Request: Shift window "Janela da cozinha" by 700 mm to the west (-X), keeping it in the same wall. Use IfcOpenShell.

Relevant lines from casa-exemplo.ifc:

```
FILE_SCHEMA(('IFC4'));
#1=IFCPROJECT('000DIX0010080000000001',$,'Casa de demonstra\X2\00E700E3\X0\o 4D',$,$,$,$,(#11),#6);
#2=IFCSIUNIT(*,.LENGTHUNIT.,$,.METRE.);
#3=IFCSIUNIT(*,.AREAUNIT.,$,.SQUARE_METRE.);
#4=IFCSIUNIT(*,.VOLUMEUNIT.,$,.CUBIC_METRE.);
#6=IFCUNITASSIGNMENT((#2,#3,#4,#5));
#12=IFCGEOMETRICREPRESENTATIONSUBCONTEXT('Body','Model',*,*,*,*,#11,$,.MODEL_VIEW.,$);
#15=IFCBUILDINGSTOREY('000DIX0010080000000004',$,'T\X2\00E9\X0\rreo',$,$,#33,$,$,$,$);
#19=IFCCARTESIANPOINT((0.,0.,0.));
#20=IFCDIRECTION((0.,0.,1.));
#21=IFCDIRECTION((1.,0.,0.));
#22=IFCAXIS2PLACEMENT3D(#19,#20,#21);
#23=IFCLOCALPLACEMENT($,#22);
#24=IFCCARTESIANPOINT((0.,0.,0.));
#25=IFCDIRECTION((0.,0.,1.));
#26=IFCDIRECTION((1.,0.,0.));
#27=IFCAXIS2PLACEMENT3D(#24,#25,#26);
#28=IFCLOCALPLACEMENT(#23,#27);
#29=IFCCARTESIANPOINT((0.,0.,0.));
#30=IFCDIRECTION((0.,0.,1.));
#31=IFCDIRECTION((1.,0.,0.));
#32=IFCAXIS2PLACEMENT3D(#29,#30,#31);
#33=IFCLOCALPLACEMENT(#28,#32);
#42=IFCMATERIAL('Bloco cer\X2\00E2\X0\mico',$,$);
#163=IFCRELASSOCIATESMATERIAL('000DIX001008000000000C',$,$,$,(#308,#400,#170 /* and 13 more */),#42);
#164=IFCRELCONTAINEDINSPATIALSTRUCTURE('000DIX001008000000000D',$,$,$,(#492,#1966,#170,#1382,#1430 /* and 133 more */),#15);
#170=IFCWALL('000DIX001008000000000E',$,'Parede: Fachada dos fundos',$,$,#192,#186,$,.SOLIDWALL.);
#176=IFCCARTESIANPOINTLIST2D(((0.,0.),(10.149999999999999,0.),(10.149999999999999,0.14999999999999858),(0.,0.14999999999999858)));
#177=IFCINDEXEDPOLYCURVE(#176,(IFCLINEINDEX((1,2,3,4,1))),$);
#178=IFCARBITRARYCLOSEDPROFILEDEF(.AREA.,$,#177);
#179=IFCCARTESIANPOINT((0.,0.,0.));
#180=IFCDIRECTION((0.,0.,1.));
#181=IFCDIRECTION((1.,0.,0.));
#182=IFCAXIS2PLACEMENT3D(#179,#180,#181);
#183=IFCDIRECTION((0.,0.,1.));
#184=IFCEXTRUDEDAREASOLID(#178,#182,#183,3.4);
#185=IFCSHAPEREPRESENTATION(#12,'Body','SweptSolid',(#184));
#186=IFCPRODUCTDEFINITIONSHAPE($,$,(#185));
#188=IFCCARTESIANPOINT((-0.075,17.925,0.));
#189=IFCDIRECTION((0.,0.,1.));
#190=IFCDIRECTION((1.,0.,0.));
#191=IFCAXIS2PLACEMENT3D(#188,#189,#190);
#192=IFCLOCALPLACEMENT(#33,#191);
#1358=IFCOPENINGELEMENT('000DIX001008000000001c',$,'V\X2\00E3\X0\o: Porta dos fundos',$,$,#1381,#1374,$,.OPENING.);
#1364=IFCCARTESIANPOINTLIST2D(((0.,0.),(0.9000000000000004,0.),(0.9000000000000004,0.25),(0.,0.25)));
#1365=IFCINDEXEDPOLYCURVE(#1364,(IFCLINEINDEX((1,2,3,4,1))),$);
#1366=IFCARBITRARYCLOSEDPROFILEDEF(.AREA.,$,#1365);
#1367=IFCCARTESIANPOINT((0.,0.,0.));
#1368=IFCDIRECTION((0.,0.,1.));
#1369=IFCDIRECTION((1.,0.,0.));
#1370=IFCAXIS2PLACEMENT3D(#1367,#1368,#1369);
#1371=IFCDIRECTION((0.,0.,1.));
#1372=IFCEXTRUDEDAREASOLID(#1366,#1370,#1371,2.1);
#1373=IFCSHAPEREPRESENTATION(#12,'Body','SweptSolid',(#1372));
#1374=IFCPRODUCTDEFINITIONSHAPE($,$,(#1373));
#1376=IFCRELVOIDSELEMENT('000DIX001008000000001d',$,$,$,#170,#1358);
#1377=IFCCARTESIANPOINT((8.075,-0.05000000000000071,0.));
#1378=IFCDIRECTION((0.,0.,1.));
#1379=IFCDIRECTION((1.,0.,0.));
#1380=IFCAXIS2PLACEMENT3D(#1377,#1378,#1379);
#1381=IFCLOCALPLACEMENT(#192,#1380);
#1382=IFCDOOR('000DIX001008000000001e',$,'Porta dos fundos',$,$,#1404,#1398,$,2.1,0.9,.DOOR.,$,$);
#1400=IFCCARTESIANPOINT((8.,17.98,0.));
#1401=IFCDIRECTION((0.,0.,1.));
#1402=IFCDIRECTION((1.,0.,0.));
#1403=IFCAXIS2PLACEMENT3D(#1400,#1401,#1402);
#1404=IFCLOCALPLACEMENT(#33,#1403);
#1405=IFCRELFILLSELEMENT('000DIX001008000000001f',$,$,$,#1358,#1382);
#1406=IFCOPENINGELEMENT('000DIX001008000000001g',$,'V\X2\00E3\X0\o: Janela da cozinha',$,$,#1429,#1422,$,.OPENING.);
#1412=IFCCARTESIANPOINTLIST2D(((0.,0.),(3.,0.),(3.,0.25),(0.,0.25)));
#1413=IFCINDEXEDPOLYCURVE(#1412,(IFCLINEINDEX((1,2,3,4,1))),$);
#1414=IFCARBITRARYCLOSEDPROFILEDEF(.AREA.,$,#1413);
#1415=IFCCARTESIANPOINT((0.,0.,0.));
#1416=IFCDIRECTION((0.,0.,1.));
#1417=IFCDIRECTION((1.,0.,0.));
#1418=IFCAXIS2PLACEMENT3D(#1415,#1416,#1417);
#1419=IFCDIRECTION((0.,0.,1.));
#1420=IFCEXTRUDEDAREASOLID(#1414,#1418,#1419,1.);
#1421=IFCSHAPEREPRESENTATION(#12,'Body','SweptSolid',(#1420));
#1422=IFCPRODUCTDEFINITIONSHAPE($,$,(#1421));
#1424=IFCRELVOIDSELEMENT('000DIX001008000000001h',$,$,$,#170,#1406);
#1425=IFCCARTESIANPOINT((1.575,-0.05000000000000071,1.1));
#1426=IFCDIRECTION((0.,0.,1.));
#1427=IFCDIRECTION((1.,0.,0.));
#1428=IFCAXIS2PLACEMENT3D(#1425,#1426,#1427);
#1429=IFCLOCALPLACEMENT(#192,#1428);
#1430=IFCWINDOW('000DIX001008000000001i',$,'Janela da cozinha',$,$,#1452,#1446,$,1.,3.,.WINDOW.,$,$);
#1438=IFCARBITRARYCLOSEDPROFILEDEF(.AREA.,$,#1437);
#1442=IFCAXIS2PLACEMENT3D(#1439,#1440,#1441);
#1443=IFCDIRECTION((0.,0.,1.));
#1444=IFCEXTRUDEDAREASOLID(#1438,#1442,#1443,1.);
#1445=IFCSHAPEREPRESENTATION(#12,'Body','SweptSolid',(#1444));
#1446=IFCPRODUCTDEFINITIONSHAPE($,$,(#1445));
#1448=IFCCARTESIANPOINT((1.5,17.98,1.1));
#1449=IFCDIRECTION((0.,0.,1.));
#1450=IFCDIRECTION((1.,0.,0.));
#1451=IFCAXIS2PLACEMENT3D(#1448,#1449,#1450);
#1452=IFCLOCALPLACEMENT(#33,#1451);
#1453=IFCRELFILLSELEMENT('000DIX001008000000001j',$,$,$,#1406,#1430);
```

```python
import ifcopenshell
import ifcopenshell.api.geometry
import ifcopenshell.util.placement

model = ifcopenshell.open("casa-exemplo.ifc")

window = model.by_guid("000DIX001008000000001i")
opening = window.FillsVoids[0].RelatingOpeningElement
wall = opening.VoidsElements[0].RelatingBuildingElement

wall_matrix = ifcopenshell.util.placement.get_local_placement(wall.ObjectPlacement)
shift = wall_matrix[:3, 0] * -0.7
before = ifcopenshell.util.placement.get_local_placement(window.ObjectPlacement)[:3, 3].copy()

# The window is not placed relative to its opening, so move both.
for product in (opening, window):
    matrix = ifcopenshell.util.placement.get_local_placement(product.ObjectPlacement)
    matrix[:3, 3] += shift
    ifcopenshell.api.geometry.edit_object_placement(model, product=product, matrix=matrix, is_si=False)

after = ifcopenshell.util.placement.get_local_placement(window.ObjectPlacement)[:3, 3]
print("window moved by", (after - before).round(3) + 0.0)

model.write("casa-exemplo_edited.ifc")
```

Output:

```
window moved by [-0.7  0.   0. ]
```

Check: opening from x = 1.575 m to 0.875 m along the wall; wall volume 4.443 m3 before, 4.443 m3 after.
